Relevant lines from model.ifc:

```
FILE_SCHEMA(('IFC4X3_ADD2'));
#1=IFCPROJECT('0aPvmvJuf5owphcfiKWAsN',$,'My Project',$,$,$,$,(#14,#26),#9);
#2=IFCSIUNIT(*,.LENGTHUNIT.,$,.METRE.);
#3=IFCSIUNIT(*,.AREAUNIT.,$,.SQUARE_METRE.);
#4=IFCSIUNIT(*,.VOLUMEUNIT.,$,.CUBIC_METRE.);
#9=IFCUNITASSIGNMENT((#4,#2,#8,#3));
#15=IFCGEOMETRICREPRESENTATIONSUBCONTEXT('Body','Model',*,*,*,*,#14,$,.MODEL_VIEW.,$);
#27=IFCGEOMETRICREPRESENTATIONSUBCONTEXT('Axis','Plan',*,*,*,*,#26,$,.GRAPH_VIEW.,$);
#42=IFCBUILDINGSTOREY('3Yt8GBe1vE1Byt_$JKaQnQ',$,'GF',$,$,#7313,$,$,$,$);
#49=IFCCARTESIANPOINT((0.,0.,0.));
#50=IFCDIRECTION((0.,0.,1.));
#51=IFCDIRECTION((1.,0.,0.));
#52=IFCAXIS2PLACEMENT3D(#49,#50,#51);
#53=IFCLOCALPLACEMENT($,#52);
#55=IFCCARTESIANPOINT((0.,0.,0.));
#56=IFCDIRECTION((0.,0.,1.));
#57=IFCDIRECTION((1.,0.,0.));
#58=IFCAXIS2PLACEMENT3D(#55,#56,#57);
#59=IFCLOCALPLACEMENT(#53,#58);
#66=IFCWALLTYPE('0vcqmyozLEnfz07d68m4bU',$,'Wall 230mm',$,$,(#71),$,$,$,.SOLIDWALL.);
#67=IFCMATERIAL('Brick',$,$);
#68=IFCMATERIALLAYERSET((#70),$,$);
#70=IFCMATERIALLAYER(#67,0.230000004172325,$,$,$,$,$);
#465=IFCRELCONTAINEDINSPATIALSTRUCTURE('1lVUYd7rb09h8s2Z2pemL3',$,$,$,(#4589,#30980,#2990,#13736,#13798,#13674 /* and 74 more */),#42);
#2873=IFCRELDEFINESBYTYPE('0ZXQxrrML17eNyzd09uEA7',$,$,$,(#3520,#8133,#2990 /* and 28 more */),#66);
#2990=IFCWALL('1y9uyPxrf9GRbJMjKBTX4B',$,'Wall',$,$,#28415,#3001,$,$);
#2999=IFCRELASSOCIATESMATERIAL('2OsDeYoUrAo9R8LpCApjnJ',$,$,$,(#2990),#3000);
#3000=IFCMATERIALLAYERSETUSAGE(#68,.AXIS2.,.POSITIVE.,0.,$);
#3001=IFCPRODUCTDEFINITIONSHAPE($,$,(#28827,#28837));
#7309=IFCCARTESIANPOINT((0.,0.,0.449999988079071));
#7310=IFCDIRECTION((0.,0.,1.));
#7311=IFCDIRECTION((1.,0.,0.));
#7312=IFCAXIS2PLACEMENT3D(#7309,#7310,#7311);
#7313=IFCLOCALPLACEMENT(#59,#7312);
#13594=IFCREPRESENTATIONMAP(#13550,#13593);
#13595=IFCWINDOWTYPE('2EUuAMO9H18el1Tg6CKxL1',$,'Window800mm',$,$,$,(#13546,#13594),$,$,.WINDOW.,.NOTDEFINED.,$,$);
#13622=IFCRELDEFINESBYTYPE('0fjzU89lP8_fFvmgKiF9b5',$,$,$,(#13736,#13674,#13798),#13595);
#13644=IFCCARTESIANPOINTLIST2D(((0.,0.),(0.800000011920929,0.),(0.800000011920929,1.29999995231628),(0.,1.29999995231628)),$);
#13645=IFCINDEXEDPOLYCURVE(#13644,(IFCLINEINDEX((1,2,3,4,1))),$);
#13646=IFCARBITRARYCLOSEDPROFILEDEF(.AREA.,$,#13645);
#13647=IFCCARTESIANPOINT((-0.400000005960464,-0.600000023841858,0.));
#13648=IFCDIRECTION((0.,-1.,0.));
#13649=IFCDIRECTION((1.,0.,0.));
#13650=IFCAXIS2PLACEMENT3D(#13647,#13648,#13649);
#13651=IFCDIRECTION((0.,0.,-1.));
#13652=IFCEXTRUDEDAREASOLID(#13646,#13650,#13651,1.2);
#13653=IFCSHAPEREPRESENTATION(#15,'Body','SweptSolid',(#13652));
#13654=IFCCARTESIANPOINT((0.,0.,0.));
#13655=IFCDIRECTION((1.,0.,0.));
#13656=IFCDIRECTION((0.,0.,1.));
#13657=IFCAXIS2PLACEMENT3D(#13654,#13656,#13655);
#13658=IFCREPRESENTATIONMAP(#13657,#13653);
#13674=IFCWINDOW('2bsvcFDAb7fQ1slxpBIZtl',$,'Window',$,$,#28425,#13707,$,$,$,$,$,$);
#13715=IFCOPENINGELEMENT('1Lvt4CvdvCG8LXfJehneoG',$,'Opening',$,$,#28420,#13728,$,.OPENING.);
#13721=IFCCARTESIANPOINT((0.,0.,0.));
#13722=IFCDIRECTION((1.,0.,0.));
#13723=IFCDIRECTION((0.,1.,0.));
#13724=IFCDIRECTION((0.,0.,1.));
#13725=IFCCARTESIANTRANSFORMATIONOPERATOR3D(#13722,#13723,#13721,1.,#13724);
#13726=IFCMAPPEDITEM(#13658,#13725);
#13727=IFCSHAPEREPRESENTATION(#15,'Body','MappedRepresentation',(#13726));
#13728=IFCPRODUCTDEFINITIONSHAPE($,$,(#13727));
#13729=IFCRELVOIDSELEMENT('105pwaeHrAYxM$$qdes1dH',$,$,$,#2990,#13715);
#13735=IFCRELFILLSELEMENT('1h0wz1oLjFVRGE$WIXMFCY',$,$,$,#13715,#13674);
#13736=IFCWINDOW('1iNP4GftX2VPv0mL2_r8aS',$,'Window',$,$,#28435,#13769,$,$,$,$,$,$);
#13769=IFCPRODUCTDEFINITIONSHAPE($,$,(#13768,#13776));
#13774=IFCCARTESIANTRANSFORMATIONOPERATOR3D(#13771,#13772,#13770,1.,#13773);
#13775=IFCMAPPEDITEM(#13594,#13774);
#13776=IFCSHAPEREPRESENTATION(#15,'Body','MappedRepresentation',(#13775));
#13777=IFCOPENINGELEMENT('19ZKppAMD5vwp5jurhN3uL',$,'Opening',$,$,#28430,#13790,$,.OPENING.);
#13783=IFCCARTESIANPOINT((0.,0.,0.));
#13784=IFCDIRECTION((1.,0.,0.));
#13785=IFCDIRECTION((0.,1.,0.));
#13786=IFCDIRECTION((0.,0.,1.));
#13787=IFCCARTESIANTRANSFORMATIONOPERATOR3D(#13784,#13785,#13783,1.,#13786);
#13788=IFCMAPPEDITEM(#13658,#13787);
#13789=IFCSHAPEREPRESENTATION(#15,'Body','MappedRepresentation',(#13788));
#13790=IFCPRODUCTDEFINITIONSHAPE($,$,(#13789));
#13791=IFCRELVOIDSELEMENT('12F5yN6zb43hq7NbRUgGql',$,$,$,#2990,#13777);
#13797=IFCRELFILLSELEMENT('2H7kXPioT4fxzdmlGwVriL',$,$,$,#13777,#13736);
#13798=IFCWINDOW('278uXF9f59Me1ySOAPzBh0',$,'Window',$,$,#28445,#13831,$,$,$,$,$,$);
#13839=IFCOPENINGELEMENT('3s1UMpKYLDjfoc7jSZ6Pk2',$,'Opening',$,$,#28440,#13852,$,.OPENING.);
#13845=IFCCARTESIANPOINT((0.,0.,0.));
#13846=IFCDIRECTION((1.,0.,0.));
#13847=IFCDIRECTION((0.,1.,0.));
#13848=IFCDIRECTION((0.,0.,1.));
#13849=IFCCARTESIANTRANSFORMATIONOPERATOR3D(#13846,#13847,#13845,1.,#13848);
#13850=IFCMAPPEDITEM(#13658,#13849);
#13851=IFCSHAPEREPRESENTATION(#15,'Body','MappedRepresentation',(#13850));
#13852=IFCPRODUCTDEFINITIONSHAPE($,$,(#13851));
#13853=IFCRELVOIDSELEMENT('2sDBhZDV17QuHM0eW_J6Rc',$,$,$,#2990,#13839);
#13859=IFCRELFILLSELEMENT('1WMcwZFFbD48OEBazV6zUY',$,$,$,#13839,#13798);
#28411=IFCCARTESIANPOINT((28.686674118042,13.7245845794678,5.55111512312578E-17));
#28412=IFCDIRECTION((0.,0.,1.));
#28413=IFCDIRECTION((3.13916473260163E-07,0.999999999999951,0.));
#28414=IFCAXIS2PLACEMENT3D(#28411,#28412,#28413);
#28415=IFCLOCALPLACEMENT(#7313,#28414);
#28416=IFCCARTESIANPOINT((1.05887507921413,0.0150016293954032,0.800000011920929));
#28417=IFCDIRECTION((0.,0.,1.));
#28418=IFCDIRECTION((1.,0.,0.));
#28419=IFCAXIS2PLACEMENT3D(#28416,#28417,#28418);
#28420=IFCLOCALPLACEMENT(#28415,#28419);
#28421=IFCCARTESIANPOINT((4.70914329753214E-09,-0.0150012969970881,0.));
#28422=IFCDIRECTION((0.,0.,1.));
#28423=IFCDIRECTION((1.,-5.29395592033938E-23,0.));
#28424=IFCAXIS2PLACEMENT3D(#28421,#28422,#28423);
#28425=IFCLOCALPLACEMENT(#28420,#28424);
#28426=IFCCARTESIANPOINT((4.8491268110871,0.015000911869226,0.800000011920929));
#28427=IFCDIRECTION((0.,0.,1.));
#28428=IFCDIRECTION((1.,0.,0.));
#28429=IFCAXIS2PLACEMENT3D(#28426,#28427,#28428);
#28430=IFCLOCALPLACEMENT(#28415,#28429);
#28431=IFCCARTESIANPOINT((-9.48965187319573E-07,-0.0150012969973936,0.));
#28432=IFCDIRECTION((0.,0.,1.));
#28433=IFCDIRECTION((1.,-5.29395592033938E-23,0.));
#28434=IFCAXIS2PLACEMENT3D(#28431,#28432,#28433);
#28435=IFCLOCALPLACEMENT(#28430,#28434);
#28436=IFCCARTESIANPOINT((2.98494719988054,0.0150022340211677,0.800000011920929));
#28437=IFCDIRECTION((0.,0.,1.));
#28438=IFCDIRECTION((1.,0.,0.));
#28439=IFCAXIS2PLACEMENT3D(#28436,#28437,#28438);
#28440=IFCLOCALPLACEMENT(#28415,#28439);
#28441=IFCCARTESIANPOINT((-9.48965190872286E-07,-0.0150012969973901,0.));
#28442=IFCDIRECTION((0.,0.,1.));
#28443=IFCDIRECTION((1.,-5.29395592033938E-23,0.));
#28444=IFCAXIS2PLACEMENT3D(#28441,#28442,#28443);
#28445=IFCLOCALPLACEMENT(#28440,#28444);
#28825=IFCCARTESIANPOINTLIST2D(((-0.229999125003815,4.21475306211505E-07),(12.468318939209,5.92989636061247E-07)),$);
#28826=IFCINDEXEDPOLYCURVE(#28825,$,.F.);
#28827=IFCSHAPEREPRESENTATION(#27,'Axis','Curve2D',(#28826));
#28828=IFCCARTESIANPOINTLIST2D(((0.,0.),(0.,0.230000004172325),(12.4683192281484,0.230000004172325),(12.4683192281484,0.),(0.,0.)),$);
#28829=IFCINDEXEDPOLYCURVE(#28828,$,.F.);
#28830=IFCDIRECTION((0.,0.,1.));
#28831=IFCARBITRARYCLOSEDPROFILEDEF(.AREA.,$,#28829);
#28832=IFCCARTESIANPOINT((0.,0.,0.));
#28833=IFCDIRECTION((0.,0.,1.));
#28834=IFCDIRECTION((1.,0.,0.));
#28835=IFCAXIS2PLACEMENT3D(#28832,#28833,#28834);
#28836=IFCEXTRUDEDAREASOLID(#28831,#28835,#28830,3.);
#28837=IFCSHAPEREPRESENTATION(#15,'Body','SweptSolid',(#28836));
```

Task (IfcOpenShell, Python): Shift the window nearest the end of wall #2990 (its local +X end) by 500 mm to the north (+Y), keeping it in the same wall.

```python
import ifcopenshell
import ifcopenshell.api.geometry
import ifcopenshell.util.placement
import ifcopenshell.util.unit

model = ifcopenshell.open("model.ifc")
unit_scale = ifcopenshell.util.unit.calculate_unit_scale(model)

window = model.by_guid("1iNP4GftX2VPv0mL2_r8aS")
opening = window.FillsVoids[0].RelatingOpeningElement
wall = opening.VoidsElements[0].RelatingBuildingElement

wall_matrix = ifcopenshell.util.placement.get_local_placement(wall.ObjectPlacement)
shift = wall_matrix[:3, 0] * 0.5 / unit_scale
before = ifcopenshell.util.placement.get_local_placement(window.ObjectPlacement)[:3, 3].copy()

# The window is placed relative to its opening, so it follows when the opening moves.
matrix = ifcopenshell.util.placement.get_local_placement(opening.ObjectPlacement)
matrix[:3, 3] += shift
ifcopenshell.api.geometry.edit_object_placement(
    model, product=opening, matrix=matrix, is_si=False, should_transform_children=True
)

after = ifcopenshell.util.placement.get_local_placement(window.ObjectPlacement)[:3, 3]
print("window moved by", (after - before).round(3) + 0.0)

model.write("model-out.ifc")
```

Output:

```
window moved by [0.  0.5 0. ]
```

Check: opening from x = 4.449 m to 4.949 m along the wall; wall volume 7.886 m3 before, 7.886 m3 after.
